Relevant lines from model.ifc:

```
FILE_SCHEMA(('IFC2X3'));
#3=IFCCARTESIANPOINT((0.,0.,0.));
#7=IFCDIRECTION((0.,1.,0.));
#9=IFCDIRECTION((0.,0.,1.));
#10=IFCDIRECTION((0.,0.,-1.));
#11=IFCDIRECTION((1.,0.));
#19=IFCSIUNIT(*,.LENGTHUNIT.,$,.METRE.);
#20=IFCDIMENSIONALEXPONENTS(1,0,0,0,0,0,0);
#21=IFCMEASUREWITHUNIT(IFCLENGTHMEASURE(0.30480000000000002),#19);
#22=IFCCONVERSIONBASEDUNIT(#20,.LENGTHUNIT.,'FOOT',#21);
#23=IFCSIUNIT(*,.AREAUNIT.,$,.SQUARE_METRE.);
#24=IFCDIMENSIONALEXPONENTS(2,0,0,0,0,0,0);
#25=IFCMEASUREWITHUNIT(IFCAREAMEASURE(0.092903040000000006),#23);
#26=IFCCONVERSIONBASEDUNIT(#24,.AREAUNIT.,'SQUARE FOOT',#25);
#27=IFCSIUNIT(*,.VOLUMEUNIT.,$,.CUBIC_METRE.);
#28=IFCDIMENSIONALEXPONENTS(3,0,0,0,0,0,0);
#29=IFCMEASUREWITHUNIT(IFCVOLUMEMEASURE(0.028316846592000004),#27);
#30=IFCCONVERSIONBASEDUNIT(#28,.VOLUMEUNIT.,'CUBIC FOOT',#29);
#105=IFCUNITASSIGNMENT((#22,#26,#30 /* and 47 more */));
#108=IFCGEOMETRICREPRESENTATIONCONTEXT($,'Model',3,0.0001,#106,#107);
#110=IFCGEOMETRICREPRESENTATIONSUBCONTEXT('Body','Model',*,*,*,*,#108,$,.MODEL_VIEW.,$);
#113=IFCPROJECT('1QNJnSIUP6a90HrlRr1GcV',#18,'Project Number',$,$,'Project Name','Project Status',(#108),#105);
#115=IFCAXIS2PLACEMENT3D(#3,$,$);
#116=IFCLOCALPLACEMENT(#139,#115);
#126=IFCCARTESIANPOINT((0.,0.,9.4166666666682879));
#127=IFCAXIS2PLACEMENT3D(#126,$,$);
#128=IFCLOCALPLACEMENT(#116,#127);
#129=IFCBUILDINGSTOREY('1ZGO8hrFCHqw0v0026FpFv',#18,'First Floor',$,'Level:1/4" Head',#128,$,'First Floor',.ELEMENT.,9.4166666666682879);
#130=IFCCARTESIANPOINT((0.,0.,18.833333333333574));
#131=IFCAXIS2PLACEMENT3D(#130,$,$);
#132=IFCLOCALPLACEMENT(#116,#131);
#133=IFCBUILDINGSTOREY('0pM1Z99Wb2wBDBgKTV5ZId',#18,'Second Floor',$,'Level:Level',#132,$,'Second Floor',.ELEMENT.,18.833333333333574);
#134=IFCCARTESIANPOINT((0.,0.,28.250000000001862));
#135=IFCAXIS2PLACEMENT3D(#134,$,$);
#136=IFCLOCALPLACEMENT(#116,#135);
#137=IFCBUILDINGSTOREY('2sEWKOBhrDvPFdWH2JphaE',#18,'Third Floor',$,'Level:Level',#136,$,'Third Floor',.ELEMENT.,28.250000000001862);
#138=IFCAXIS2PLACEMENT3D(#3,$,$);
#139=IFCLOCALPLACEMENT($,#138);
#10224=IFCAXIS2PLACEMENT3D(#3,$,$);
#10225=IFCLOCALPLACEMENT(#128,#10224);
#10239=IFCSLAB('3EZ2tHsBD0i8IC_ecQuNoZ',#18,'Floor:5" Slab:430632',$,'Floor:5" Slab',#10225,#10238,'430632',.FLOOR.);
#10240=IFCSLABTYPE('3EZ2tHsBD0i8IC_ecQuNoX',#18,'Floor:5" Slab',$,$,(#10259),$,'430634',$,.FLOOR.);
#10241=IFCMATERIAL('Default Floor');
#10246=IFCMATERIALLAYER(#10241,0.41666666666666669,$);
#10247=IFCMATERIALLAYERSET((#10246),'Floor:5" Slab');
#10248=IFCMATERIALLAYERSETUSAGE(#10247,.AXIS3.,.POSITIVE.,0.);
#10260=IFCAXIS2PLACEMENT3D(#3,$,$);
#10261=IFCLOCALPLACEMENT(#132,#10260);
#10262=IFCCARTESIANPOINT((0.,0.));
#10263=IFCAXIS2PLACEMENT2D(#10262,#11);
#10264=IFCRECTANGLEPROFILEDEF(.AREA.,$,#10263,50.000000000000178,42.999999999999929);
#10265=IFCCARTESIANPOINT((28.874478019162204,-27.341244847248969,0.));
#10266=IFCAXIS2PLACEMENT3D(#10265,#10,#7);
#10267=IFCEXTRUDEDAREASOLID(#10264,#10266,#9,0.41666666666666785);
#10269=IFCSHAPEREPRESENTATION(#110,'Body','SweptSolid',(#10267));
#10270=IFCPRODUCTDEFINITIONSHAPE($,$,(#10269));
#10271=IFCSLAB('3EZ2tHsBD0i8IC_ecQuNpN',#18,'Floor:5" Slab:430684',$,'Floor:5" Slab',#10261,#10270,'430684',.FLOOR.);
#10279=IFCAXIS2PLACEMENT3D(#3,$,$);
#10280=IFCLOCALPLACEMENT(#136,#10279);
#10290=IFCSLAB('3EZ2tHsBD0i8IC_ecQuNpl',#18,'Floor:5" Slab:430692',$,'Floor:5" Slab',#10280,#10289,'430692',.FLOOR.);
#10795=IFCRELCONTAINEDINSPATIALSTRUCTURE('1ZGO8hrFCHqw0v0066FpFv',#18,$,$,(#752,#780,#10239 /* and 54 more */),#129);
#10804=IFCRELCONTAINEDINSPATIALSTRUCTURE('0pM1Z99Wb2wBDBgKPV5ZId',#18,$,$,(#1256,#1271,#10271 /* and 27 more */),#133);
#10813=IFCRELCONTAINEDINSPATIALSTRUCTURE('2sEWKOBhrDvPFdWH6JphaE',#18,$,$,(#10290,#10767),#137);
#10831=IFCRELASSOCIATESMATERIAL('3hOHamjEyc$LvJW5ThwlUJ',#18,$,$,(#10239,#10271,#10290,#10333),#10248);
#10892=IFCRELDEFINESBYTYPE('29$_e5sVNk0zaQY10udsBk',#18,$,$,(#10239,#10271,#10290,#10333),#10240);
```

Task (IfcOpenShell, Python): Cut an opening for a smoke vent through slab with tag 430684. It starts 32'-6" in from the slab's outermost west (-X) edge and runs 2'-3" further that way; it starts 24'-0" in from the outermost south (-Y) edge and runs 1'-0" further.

```python
import numpy as np
import ifcopenshell
import ifcopenshell.api.feature
import ifcopenshell.api.geometry
import ifcopenshell.api.root
import ifcopenshell.geom
import ifcopenshell.util.placement
import ifcopenshell.util.representation
import ifcopenshell.util.shape
import ifcopenshell.util.unit

model = ifcopenshell.open("model.ifc")
unit_scale = ifcopenshell.util.unit.calculate_unit_scale(model)
settings = ifcopenshell.geom.settings()


def volume(element):
    """Net volume in cubic metres, openings subtracted."""
    shape = ifcopenshell.geom.create_shape(settings, element)
    return ifcopenshell.util.shape.get_volume(shape.geometry)


slab = model.by_guid("3EZ2tHsBD0i8IC_ecQuNpN")
before = volume(slab)

# Extent in the slab's own axes, in metres. The edges named are its -X and -Y sides.
slab_shape = ifcopenshell.geom.create_shape(settings, slab)
vertices = ifcopenshell.util.shape.get_vertices(slab_shape.geometry)
x_min, y_min, bottom = vertices.min(axis=0)
top = vertices[:, 2].max()

opening = ifcopenshell.api.root.create_entity(model, ifc_class="IfcOpeningElement", name="Smoke vent opening")
context = ifcopenshell.util.representation.get_context(model, "Model", "Body", "MODEL_VIEW")
width, depth = 0.6858, 0.3048
outline = [(0.0, 0.0), (width, 0.0), (width, depth), (0.0, depth), (0.0, 0.0)]
# Overshoot both faces by 50 mm so the cut is clean.
shape = ifcopenshell.api.geometry.add_slab_representation(
    model, context=context, depth=top - bottom + 0.1, polyline=outline
)
ifcopenshell.api.geometry.assign_representation(model, product=opening, representation=shape)

matrix = ifcopenshell.util.placement.get_local_placement(slab.ObjectPlacement)
matrix[:, 3] = matrix @ np.append(np.array([x_min + 9.906, y_min + 7.3152, bottom - 0.05]) / unit_scale, 1.0)
ifcopenshell.api.geometry.edit_object_placement(model, product=opening, matrix=matrix, is_si=False)
ifcopenshell.api.feature.add_feature(model, feature=opening, element=slab)

after = volume(slab)

print(f"slab volume {before:.3f} -> {after:.3f} m3")

model.write("model-out.ifc")
```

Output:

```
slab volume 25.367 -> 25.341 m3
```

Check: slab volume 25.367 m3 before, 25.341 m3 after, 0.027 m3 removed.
